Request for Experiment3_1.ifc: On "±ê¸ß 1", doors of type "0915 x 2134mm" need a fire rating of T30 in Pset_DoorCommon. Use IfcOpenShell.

First a look at what the model holds.

```python
import ifcopenshell
import ifcopenshell.util.element

model = ifcopenshell.open("Experiment3_1.ifc")
print(model.schema)
storey = next(s for s in model.by_type("IfcBuildingStorey") if s.Name == "±ê¸ß 1")
doors = [e for e in ifcopenshell.util.element.get_decomposition(storey) if e.is_a("IfcDoor")]
seen = {}
for e in doors:
    element_type = ifcopenshell.util.element.get_type(e)
    key = (element_type.Name if element_type != e and element_type else None, ifcopenshell.util.element.get_pset(e, "Pset_DoorCommon", "FireRating"))
    seen[key] = seen.get(key, 0) + 1
for (name, value), count in sorted(seen.items(), key=str):
    print(count, "x", name, "|", value)
```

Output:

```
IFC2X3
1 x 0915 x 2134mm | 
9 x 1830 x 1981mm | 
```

```python
import ifcopenshell
import ifcopenshell.api.pset
import ifcopenshell.util.element

model = ifcopenshell.open("Experiment3_1.ifc")

storey = next(s for s in model.by_type("IfcBuildingStorey") if s.Name == "±ê¸ß 1")
doors = [e for e in ifcopenshell.util.element.get_decomposition(storey) if e.is_a("IfcDoor")]

count = 0
for e in doors:
    element_type = ifcopenshell.util.element.get_type(e)
    if element_type in (None, e) or element_type.Name != "0915 x 2134mm":
        continue
    # add_pset returns the element's existing set when there is one.
    pset = ifcopenshell.api.pset.add_pset(model, product=e, name="Pset_DoorCommon")
    ifcopenshell.api.pset.edit_pset(model, pset=pset, properties={"FireRating": "T30"})
    count += 1

print(count, "doors updated")

model.write("Experiment3_1_updated.ifc")
```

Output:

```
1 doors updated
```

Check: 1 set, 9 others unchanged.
